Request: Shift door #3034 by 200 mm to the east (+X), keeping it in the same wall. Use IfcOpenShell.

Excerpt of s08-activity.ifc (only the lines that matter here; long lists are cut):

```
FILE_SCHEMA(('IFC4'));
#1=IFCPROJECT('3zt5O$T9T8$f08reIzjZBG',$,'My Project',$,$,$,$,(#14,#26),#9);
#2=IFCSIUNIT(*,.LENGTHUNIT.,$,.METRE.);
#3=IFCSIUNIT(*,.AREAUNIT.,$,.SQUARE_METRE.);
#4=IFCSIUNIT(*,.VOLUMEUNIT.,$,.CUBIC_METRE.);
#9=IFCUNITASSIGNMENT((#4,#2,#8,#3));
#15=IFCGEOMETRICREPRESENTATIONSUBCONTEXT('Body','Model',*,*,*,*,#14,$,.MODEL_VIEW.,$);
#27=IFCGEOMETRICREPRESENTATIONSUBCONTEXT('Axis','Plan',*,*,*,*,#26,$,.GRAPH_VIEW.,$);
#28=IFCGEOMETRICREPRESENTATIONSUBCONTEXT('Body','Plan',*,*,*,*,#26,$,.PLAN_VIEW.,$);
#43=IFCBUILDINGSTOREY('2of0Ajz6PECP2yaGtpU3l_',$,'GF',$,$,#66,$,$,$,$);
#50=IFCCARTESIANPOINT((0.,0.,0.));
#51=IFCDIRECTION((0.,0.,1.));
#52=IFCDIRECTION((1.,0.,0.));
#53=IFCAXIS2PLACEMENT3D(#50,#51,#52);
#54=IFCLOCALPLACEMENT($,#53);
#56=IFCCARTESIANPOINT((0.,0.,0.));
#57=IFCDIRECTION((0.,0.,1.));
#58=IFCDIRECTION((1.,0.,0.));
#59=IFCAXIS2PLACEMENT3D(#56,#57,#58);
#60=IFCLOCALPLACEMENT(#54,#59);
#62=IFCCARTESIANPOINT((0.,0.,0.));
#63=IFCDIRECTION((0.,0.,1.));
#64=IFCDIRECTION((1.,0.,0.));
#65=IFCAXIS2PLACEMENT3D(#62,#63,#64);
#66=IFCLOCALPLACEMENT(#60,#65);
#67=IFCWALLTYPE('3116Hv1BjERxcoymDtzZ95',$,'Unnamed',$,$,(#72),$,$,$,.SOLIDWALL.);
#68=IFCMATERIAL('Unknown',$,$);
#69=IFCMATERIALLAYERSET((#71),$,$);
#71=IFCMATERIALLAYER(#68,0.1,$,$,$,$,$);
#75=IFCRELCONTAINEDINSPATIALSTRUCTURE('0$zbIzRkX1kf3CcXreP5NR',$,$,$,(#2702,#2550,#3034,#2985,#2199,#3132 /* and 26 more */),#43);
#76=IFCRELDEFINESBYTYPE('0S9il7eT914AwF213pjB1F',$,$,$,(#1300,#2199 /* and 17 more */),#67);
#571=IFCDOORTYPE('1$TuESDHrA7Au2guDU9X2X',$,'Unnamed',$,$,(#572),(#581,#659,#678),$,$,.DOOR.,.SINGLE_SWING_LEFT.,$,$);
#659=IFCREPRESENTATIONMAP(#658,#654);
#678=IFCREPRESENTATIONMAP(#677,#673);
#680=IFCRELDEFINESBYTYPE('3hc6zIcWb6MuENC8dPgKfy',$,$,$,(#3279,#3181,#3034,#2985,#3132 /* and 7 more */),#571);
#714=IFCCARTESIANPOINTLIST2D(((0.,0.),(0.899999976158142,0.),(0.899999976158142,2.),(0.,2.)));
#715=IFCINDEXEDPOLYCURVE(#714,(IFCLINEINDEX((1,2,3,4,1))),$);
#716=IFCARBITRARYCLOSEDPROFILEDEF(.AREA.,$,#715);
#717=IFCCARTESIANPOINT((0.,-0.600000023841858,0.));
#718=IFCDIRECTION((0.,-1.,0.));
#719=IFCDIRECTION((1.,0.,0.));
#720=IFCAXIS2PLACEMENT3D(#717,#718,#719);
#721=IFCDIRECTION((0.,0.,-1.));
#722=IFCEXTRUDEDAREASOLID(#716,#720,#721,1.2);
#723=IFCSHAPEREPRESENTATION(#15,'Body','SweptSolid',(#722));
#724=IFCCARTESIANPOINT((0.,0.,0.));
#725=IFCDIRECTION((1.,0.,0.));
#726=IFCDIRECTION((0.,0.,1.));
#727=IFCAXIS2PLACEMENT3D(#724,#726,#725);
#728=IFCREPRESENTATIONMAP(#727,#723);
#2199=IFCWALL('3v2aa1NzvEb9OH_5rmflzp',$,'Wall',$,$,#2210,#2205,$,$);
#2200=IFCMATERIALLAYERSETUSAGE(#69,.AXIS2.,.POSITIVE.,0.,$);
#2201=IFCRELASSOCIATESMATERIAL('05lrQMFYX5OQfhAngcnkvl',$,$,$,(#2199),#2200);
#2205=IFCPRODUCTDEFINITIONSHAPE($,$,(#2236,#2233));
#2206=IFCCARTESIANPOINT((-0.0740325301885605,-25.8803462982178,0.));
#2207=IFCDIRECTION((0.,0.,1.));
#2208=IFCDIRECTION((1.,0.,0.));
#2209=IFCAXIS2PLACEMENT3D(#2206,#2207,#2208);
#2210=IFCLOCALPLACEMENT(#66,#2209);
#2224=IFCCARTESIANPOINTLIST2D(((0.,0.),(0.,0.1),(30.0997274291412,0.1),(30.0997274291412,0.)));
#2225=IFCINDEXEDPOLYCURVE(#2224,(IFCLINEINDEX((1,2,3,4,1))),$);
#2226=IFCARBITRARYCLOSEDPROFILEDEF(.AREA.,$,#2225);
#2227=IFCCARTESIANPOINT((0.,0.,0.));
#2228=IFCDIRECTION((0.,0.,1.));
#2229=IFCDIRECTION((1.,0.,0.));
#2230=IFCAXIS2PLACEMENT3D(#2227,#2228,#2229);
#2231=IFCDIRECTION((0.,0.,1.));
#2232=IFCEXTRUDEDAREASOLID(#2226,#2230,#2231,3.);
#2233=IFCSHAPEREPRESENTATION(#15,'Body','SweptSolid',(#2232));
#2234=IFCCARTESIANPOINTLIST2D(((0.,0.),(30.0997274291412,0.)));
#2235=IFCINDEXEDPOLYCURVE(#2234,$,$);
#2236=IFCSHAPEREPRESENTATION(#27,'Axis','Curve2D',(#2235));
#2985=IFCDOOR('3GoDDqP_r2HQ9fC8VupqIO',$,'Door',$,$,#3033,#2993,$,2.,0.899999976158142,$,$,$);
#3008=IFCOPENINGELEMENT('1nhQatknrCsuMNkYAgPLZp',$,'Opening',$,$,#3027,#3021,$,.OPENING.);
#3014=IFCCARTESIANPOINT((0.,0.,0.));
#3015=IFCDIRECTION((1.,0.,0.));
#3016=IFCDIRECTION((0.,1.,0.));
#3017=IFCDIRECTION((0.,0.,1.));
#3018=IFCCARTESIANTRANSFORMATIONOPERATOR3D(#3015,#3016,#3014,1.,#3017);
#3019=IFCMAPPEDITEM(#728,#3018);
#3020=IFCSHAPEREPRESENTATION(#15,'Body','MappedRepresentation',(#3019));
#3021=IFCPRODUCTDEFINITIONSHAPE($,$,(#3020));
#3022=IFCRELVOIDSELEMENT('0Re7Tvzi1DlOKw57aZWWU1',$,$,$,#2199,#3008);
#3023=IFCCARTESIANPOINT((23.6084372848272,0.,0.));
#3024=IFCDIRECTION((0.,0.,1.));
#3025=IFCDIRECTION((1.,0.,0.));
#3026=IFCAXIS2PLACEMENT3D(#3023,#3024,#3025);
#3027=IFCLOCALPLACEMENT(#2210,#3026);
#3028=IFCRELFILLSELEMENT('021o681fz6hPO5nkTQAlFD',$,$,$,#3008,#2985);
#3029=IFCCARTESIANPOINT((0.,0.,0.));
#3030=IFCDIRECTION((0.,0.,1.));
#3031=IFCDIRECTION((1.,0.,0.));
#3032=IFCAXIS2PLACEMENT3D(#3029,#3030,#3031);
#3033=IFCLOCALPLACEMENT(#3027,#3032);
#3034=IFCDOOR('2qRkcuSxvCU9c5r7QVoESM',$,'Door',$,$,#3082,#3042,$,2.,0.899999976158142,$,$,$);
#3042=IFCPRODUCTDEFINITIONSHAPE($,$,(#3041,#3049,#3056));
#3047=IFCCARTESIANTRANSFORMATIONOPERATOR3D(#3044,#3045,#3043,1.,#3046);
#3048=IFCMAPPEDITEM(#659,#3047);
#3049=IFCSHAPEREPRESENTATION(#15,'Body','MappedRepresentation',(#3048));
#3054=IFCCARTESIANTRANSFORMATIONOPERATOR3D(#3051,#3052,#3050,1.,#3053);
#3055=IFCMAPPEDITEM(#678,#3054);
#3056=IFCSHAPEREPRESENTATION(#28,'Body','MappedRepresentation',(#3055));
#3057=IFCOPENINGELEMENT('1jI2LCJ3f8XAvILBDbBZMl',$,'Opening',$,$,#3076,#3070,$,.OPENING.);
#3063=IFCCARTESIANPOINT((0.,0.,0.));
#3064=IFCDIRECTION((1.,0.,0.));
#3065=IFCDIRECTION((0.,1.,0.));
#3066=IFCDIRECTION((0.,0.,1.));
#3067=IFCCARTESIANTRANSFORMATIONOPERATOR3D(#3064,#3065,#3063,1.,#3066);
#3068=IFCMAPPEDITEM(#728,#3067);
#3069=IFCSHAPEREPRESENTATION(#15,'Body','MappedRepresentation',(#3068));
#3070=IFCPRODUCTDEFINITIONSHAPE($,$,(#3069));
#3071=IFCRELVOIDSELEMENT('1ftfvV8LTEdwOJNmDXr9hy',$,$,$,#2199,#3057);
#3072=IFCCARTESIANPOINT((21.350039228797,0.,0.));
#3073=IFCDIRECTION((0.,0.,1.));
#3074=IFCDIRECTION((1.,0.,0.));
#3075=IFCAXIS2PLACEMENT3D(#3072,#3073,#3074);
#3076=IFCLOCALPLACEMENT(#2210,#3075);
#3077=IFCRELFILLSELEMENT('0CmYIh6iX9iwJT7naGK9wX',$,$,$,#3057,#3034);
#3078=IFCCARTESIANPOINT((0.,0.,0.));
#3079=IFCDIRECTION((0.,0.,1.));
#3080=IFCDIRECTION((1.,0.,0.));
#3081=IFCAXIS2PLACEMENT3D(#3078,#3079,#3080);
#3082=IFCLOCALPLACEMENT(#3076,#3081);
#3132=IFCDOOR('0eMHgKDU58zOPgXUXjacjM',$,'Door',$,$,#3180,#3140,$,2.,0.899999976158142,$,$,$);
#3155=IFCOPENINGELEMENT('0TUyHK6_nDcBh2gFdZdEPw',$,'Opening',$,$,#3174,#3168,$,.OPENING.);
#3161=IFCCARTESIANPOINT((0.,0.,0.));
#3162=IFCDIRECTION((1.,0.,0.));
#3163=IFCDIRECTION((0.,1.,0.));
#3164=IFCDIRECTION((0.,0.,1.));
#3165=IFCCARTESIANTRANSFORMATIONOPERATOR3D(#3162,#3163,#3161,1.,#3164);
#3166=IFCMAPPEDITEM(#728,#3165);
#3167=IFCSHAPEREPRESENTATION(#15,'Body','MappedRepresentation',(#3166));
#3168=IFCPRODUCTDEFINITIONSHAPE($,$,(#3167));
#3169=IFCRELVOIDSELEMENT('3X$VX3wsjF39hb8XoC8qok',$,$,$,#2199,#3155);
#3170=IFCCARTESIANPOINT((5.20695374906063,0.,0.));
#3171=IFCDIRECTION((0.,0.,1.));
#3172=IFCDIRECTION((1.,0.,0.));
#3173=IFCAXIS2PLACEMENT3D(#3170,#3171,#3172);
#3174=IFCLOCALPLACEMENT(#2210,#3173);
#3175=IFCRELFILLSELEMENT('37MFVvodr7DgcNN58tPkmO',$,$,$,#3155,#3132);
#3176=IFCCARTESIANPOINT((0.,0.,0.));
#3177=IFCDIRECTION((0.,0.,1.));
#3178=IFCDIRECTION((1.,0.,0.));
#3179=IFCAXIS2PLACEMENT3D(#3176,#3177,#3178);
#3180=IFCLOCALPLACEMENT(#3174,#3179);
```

```python
import ifcopenshell
import ifcopenshell.api.geometry
import ifcopenshell.util.placement
import ifcopenshell.util.unit

model = ifcopenshell.open("s08-activity.ifc")
unit_scale = ifcopenshell.util.unit.calculate_unit_scale(model)

door = model.by_guid("2qRkcuSxvCU9c5r7QVoESM")
opening = door.FillsVoids[0].RelatingOpeningElement
wall = opening.VoidsElements[0].RelatingBuildingElement

wall_matrix = ifcopenshell.util.placement.get_local_placement(wall.ObjectPlacement)
shift = wall_matrix[:3, 0] * 0.2 / unit_scale
before = ifcopenshell.util.placement.get_local_placement(door.ObjectPlacement)[:3, 3].copy()

# The door is placed relative to its opening, so it follows when the opening moves.
matrix = ifcopenshell.util.placement.get_local_placement(opening.ObjectPlacement)
matrix[:3, 3] += shift
ifcopenshell.api.geometry.edit_object_placement(
    model, product=opening, matrix=matrix, is_si=False, should_transform_children=True
)

after = ifcopenshell.util.placement.get_local_placement(door.ObjectPlacement)[:3, 3]
print("door moved by", (after - before).round(3) + 0.0)

model.write("s08-activity-out.ifc")
```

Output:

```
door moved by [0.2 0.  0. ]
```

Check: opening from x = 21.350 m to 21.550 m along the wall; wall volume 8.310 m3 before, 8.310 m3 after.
